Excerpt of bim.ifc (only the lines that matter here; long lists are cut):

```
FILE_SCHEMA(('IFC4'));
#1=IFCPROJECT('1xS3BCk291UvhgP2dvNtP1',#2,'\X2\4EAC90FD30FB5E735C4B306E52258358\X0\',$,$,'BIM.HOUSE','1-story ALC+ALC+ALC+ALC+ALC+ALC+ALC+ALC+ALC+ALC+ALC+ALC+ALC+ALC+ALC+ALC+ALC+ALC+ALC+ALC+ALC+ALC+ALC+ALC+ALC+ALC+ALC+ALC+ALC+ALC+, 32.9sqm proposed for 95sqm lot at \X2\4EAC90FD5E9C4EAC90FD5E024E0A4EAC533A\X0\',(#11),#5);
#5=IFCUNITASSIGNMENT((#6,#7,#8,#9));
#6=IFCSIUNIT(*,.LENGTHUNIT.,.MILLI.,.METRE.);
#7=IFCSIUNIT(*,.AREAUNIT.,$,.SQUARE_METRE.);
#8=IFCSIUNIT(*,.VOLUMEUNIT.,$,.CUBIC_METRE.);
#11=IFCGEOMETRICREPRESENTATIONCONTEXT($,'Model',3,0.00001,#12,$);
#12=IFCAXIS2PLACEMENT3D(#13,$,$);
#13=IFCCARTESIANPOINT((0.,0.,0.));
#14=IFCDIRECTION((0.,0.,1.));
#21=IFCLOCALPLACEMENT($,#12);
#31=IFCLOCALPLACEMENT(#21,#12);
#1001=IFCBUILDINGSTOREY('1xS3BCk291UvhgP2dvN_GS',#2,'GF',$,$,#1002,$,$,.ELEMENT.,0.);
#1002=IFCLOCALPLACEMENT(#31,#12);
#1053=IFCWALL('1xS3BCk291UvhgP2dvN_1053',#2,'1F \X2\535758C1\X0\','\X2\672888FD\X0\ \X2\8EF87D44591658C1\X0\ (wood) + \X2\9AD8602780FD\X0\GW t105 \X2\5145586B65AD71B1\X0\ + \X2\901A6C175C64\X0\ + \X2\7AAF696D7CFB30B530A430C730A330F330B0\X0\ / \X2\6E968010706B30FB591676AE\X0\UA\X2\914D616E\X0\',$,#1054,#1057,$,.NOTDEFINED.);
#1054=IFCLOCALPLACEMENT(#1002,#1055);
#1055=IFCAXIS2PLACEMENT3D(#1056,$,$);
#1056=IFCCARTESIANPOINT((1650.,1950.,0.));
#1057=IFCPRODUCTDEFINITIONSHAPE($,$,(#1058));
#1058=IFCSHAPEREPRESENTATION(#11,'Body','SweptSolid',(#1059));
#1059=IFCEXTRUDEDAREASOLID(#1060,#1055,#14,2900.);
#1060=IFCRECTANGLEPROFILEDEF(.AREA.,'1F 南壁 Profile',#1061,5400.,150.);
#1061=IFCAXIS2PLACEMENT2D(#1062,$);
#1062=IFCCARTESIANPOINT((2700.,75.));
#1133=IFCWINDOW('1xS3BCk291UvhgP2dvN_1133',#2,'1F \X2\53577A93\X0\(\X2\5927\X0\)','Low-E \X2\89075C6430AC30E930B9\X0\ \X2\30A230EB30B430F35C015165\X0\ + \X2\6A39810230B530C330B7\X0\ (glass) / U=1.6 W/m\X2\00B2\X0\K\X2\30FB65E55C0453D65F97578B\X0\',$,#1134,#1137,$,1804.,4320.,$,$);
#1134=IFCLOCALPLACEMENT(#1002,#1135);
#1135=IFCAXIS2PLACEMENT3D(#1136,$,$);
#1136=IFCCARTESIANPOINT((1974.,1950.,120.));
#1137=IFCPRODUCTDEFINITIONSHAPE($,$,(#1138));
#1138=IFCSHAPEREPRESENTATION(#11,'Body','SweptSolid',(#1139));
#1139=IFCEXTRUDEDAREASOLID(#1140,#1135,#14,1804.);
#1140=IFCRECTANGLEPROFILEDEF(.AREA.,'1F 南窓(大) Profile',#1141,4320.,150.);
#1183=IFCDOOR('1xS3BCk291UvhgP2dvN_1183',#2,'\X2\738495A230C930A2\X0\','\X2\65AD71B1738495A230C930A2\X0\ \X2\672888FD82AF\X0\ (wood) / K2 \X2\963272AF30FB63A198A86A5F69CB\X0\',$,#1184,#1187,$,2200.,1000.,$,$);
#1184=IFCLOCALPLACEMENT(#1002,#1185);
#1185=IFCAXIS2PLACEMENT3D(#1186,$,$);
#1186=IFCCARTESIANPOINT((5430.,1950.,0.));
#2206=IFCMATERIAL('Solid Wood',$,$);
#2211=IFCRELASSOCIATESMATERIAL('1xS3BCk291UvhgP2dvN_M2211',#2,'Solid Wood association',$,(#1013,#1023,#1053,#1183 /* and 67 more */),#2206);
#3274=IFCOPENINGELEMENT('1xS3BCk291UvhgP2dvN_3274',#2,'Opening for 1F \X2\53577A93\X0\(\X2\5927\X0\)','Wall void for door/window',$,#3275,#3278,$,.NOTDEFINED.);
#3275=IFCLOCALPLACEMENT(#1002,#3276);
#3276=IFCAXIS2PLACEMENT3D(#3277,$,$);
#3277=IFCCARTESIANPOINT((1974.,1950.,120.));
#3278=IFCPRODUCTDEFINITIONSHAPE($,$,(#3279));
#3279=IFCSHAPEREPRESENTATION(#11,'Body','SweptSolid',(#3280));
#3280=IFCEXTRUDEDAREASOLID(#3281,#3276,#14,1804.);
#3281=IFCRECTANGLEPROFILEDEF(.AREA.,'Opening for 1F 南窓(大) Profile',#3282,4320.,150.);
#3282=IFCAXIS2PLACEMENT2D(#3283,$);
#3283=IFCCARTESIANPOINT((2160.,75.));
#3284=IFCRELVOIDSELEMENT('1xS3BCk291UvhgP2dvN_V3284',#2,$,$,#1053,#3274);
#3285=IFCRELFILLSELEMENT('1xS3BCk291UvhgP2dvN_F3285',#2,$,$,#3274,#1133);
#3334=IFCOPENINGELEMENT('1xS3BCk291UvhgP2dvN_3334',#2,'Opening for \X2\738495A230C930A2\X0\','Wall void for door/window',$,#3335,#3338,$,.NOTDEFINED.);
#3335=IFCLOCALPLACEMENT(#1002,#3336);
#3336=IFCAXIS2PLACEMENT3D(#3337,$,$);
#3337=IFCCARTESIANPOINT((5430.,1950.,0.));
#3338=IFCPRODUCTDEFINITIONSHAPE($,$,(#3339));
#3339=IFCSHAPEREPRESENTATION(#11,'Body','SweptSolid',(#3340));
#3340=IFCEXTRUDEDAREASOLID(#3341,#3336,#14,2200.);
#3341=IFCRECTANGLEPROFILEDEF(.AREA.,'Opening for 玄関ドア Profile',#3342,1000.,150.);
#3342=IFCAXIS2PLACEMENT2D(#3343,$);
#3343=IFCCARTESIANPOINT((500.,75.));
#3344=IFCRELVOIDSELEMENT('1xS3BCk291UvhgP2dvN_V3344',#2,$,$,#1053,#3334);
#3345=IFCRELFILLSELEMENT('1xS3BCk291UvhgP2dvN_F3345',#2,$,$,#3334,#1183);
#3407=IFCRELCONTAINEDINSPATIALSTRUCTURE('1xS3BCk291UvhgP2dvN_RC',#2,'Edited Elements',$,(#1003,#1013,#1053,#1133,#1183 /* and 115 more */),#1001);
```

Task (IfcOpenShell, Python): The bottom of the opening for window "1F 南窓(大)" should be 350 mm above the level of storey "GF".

```python
import numpy as np
import ifcopenshell
import ifcopenshell.api.geometry
import ifcopenshell.geom
import ifcopenshell.util.element
import ifcopenshell.util.placement
import ifcopenshell.util.shape
import ifcopenshell.util.unit

model = ifcopenshell.open("bim.ifc")
unit_scale = ifcopenshell.util.unit.calculate_unit_scale(model)

window = model.by_id(1133)
opening = window.FillsVoids[0].RelatingOpeningElement
storey = ifcopenshell.util.element.get_container(window, ifc_class="IfcBuildingStorey")
level = ifcopenshell.util.placement.get_local_placement(storey.ObjectPlacement)[2, 3]

# The opening's origin need not be at the sill, so measure its lowest point.
shape = ifcopenshell.geom.create_shape(ifcopenshell.geom.settings(), opening)
bottom = ifcopenshell.util.shape.get_shape_bottom_elevation(shape, shape.geometry) / unit_scale
dz = level + 0.35 / unit_scale - bottom

shift = np.array([0.0, 0.0, dz])
# The window is not placed relative to its opening, so move both.
for product in (opening, window):
    matrix = ifcopenshell.util.placement.get_local_placement(product.ObjectPlacement)
    matrix[:3, 3] += shift
    ifcopenshell.api.geometry.edit_object_placement(model, product=product, matrix=matrix, is_si=False)

print(f"moved by {dz * unit_scale:+.3f} m")

model.write("bim_v2.ifc")
```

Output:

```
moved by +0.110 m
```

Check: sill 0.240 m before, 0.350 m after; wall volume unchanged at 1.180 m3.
